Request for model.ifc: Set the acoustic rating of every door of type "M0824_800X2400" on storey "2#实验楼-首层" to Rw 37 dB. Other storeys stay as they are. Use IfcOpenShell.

First a look at what the model holds.

```python
import ifcopenshell
import ifcopenshell.util.element

model = ifcopenshell.open("model.ifc")
print(model.schema)
storey = next(s for s in model.by_type("IfcBuildingStorey") if s.Name == "2#实验楼-首层")
doors = [e for e in ifcopenshell.util.element.get_decomposition(storey) if e.is_a("IfcDoor")]
seen = {}
for e in doors:
    element_type = ifcopenshell.util.element.get_type(e)
    key = (element_type.Name if element_type != e and element_type else None, ifcopenshell.util.element.get_pset(e, "Pset_DoorCommon", "AcousticRating"))
    seen[key] = seen.get(key, 0) + 1
for (name, value), count in sorted(seen.items(), key=str):
    print(count, "x", name, "|", value)
```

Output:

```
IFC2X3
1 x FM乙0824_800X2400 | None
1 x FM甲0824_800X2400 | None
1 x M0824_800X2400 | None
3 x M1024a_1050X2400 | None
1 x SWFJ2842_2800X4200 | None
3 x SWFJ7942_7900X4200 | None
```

```python
import ifcopenshell
import ifcopenshell.api.pset
import ifcopenshell.util.element

model = ifcopenshell.open("model.ifc")

storey = next(s for s in model.by_type("IfcBuildingStorey") if s.Name == "2#实验楼-首层")
doors = [e for e in ifcopenshell.util.element.get_decomposition(storey) if e.is_a("IfcDoor")]

count = 0
for e in doors:
    element_type = ifcopenshell.util.element.get_type(e)
    if element_type in (None, e) or element_type.Name != "M0824_800X2400":
        continue
    # add_pset returns the element's existing set when there is one.
    pset = ifcopenshell.api.pset.add_pset(model, product=e, name="Pset_DoorCommon")
    ifcopenshell.api.pset.edit_pset(model, pset=pset, properties={"AcousticRating": "Rw 37 dB"})
    count += 1

print(count, "doors updated")

model.write("model_v2.ifc")
```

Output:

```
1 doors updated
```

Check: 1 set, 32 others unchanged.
